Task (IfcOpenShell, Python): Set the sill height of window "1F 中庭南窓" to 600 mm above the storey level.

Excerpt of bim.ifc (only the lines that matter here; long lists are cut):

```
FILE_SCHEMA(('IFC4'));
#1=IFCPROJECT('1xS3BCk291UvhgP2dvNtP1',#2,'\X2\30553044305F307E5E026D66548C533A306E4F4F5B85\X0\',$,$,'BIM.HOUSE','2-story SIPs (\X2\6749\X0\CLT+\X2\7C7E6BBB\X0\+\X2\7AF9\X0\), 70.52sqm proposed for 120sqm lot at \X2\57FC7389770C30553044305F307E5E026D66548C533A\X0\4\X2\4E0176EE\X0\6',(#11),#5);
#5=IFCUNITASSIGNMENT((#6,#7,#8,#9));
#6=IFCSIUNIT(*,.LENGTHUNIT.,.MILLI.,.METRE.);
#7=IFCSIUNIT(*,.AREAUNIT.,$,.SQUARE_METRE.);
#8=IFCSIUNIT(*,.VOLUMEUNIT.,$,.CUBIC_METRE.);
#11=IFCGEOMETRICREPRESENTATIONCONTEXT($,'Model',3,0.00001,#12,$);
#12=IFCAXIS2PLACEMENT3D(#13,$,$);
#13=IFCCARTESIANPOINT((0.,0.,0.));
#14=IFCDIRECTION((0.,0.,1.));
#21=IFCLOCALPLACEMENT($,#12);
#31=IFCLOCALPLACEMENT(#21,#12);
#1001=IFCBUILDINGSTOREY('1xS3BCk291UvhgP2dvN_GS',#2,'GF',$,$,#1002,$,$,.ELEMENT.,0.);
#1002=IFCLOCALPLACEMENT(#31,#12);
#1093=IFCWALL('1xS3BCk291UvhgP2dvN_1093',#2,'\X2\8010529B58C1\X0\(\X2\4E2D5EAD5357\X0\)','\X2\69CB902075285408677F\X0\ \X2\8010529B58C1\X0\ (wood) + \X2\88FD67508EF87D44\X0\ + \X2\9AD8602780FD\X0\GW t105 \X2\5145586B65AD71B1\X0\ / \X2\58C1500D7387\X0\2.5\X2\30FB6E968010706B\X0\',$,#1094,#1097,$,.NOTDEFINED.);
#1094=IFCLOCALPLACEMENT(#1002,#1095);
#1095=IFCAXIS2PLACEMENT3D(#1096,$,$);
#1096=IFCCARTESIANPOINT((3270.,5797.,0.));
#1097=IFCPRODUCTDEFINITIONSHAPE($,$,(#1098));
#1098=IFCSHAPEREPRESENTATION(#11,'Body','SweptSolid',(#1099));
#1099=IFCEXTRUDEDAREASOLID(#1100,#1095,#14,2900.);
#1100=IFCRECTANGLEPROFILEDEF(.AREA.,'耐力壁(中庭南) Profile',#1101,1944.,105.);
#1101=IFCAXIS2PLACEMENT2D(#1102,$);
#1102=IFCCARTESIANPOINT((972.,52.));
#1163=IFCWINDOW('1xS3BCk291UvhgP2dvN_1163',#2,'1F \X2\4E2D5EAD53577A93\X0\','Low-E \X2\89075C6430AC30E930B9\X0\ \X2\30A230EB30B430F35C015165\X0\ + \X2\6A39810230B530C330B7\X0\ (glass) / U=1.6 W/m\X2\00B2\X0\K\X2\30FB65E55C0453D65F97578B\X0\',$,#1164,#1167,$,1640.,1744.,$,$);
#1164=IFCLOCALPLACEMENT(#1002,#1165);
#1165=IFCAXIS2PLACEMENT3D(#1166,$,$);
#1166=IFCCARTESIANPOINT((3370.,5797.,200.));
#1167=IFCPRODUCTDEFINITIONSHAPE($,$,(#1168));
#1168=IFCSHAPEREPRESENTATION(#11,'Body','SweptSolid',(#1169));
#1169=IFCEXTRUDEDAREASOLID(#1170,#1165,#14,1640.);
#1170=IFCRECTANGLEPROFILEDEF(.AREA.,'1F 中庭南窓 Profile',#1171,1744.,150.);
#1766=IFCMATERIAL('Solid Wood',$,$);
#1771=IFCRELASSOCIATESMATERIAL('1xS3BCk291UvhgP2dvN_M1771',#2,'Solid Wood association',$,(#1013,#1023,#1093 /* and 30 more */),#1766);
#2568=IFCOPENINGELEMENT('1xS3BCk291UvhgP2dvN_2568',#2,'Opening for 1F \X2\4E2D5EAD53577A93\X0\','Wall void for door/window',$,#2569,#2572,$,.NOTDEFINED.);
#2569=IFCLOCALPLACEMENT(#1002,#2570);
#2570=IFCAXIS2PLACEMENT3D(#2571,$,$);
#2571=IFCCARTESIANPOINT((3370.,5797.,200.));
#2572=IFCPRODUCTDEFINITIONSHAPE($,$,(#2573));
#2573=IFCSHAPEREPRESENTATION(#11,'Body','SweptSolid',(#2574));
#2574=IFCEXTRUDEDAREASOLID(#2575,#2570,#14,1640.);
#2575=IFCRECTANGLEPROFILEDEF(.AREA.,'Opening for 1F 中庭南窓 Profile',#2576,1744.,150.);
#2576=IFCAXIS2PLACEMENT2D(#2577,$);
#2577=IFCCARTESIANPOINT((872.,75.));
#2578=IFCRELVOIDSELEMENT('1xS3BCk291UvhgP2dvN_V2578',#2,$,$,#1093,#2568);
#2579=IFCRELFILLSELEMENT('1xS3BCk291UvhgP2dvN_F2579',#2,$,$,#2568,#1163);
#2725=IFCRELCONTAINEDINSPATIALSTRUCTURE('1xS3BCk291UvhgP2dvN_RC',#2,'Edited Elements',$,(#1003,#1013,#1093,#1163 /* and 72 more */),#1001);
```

```python
import numpy as np
import ifcopenshell
import ifcopenshell.api.geometry
import ifcopenshell.geom
import ifcopenshell.util.element
import ifcopenshell.util.placement
import ifcopenshell.util.shape
import ifcopenshell.util.unit

model = ifcopenshell.open("bim.ifc")
unit_scale = ifcopenshell.util.unit.calculate_unit_scale(model)

window = model.by_id(1163)
opening = window.FillsVoids[0].RelatingOpeningElement
storey = ifcopenshell.util.element.get_container(window, ifc_class="IfcBuildingStorey")
level = ifcopenshell.util.placement.get_local_placement(storey.ObjectPlacement)[2, 3]

# The opening's origin need not be at the sill, so measure its lowest point.
shape = ifcopenshell.geom.create_shape(ifcopenshell.geom.settings(), opening)
bottom = ifcopenshell.util.shape.get_shape_bottom_elevation(shape, shape.geometry) / unit_scale
dz = level + 0.6 / unit_scale - bottom

shift = np.array([0.0, 0.0, dz])
# The window is not placed relative to its opening, so move both.
for product in (opening, window):
    matrix = ifcopenshell.util.placement.get_local_placement(product.ObjectPlacement)
    matrix[:3, 3] += shift
    ifcopenshell.api.geometry.edit_object_placement(model, product=product, matrix=matrix, is_si=False)

print(f"moved by {dz * unit_scale:+.3f} m")

model.write("bim_rev.ifc")
```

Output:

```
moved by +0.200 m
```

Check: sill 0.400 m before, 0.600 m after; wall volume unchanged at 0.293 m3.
